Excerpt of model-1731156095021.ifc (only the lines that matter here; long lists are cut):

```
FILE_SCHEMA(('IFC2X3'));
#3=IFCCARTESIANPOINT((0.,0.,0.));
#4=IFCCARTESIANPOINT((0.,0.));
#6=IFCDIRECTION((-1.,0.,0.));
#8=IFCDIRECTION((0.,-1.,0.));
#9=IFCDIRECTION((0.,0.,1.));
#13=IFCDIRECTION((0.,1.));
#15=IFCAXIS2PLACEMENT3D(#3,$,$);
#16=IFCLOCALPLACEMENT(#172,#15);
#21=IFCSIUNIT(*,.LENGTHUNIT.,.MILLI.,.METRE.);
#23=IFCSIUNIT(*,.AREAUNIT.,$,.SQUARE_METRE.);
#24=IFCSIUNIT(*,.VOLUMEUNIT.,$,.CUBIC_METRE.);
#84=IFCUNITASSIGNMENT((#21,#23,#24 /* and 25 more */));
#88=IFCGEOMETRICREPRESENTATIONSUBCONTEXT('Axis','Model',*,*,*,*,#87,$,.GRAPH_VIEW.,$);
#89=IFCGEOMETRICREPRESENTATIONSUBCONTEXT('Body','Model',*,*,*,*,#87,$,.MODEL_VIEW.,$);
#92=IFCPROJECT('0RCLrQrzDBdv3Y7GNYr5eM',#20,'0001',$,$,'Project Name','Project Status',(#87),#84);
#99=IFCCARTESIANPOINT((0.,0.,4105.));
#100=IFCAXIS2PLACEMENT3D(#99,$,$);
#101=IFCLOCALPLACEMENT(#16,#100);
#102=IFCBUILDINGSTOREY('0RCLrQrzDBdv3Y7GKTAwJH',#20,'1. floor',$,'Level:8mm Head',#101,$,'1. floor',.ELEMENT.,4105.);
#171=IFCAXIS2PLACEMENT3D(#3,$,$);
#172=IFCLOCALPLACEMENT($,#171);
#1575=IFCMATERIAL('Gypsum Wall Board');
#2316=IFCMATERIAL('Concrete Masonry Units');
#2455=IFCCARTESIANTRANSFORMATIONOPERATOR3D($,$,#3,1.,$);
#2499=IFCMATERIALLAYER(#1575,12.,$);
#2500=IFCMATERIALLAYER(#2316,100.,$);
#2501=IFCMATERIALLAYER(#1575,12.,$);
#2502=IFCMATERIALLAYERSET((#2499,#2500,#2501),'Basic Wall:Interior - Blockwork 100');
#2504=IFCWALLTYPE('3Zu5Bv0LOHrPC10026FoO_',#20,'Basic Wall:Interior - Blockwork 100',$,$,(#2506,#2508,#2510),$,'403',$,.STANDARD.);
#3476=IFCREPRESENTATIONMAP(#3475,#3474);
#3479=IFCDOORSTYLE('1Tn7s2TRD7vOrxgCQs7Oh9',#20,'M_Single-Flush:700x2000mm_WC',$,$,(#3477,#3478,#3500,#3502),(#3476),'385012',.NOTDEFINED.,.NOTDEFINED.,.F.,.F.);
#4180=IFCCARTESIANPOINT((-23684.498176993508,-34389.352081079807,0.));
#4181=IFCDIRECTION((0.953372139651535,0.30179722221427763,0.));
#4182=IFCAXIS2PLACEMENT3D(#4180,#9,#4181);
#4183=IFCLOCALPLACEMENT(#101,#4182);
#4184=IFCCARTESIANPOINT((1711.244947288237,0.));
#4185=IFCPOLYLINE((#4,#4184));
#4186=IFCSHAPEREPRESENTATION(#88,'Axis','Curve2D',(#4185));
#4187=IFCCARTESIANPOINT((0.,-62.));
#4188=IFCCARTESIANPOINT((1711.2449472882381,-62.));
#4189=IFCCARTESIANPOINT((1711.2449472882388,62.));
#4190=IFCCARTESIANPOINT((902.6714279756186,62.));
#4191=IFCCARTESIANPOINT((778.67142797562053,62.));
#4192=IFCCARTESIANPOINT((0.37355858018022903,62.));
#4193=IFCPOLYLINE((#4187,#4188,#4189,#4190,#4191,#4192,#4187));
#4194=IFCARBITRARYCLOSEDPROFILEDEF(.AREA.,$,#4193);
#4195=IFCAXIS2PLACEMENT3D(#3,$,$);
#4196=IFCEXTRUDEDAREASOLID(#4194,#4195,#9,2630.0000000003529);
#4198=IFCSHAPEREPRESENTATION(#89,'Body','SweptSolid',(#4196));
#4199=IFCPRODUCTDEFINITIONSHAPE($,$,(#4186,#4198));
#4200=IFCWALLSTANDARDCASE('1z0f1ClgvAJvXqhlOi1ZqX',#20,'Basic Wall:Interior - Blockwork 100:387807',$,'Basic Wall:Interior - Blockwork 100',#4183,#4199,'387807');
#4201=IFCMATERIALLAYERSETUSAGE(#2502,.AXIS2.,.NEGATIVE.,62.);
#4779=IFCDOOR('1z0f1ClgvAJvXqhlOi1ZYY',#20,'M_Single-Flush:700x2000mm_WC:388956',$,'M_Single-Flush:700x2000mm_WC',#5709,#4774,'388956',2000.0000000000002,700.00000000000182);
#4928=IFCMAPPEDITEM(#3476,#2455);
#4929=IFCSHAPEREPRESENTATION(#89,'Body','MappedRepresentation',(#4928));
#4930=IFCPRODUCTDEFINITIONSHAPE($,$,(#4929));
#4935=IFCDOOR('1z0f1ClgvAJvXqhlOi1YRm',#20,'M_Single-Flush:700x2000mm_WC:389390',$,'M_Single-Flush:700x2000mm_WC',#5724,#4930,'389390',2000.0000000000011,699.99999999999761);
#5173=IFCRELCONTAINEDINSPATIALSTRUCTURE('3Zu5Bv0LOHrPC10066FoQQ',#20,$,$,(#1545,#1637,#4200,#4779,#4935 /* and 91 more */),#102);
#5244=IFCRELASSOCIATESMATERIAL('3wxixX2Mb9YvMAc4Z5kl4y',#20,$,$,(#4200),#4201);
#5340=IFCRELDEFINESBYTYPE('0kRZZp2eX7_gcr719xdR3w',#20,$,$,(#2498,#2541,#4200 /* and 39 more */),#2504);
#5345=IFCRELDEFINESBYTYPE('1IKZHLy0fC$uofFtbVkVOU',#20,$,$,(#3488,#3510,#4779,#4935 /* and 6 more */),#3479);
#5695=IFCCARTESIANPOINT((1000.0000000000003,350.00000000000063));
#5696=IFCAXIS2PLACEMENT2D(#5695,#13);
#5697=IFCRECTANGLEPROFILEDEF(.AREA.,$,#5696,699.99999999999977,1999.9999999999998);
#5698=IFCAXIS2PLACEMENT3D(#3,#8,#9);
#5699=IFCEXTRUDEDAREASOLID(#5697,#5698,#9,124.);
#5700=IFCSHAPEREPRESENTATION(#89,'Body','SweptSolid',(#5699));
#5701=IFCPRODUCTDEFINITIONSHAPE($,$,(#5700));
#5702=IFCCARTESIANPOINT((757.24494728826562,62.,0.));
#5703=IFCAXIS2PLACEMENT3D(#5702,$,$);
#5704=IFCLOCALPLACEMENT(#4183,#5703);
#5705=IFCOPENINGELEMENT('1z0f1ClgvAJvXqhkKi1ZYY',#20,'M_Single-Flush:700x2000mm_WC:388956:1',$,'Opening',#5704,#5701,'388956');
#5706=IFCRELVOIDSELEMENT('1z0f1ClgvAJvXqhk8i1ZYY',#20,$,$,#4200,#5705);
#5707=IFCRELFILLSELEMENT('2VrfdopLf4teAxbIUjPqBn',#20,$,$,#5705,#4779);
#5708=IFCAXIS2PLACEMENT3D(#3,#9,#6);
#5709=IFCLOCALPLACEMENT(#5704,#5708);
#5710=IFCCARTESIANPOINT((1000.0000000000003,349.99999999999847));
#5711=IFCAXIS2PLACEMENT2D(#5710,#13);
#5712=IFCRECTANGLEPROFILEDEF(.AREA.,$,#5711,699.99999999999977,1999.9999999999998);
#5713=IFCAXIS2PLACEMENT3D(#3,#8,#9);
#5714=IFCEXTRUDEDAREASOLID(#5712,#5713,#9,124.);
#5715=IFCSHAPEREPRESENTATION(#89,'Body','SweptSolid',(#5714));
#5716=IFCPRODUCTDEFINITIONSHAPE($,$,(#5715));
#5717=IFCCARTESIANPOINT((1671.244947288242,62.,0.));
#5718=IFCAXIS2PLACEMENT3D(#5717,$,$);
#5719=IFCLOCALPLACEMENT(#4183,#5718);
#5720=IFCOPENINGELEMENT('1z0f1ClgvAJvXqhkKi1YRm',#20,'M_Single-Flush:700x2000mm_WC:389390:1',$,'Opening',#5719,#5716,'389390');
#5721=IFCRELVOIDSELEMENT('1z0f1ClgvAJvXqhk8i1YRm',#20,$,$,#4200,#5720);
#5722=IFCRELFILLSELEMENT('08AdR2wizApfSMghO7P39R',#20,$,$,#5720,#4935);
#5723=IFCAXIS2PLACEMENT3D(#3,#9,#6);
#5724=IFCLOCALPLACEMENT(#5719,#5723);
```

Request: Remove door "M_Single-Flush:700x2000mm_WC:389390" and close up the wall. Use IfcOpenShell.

```python
import ifcopenshell
import ifcopenshell.api.feature
import ifcopenshell.api.root
import ifcopenshell.geom
import ifcopenshell.util.shape

model = ifcopenshell.open("model-1731156095021.ifc")
settings = ifcopenshell.geom.settings()


def volume(element):
    """Net volume in cubic metres, openings subtracted."""
    shape = ifcopenshell.geom.create_shape(settings, element)
    return ifcopenshell.util.shape.get_volume(shape.geometry)


door = model.by_id(4935)
opening = door.FillsVoids[0].RelatingOpeningElement
wall = opening.VoidsElements[0].RelatingBuildingElement
before = volume(wall)

ifcopenshell.api.root.remove_product(model, product=door)
ifcopenshell.api.feature.remove_feature(model, feature=opening)

after = volume(wall)

print(f"wall volume {before:.3f} -> {after:.3f} m3")

model.write("model-1731156095021_edited.ifc")
```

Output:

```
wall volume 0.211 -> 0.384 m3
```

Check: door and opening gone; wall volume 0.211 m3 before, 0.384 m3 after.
